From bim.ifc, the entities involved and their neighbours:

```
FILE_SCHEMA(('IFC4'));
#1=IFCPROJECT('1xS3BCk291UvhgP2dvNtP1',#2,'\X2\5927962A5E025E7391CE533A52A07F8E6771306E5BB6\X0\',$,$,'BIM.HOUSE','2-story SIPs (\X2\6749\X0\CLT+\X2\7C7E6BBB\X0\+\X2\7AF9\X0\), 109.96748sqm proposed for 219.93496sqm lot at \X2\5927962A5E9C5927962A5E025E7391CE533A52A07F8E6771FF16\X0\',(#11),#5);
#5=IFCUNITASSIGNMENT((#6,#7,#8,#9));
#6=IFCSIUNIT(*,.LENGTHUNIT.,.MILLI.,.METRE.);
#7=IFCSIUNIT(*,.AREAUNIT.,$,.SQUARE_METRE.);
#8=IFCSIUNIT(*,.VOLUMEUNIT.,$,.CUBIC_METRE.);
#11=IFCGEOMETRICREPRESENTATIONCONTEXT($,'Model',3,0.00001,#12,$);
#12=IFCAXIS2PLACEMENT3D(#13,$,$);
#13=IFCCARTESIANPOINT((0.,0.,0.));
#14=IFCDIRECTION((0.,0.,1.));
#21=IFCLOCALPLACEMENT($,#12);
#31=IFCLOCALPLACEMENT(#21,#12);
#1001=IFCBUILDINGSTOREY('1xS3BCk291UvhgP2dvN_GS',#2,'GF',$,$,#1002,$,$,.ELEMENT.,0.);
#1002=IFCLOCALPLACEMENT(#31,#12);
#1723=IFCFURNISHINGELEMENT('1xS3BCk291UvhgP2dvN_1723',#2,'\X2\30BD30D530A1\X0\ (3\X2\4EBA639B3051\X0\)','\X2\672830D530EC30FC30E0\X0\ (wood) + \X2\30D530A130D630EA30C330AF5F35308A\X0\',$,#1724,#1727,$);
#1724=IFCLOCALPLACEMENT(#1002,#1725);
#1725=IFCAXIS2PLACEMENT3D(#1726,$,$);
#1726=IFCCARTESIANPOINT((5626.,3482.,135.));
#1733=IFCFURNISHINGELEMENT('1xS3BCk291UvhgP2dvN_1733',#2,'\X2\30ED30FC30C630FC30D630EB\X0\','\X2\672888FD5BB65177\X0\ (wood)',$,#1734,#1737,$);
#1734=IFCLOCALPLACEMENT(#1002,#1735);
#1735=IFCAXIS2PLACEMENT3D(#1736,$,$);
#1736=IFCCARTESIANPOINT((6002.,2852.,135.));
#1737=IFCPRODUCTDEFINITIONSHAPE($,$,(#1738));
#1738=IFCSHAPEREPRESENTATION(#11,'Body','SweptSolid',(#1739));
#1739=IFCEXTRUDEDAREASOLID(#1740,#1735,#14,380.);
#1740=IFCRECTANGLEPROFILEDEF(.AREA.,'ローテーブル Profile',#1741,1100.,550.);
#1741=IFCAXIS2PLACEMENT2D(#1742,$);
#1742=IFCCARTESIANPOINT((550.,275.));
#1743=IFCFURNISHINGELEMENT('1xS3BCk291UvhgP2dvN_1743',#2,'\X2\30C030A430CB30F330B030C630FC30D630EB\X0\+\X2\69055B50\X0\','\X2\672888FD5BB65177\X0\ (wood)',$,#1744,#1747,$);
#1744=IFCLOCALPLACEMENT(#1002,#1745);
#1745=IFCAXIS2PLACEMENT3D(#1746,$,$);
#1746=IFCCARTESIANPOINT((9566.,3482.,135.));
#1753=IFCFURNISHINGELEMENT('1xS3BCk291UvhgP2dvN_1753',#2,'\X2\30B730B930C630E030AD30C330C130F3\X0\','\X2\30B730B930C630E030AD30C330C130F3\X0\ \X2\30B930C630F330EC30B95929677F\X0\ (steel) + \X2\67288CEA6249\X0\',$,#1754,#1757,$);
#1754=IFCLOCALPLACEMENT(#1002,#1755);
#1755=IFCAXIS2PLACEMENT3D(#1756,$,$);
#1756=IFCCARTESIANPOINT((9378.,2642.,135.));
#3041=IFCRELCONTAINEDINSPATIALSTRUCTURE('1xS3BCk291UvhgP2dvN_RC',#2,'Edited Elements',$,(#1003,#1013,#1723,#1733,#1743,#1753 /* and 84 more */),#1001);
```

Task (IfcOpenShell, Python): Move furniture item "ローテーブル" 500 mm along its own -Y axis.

```python
import ifcopenshell
import ifcopenshell.api.geometry
import ifcopenshell.util.placement
import ifcopenshell.util.unit

model = ifcopenshell.open("bim.ifc")
unit_scale = ifcopenshell.util.unit.calculate_unit_scale(model)

item = model.by_guid("1xS3BCk291UvhgP2dvN_1733")
matrix = ifcopenshell.util.placement.get_local_placement(item.ObjectPlacement)
matrix[:3, 3] -= matrix[:3, 1] * 0.5 / unit_scale
ifcopenshell.api.geometry.edit_object_placement(model, product=item, matrix=matrix, is_si=False)

print(ifcopenshell.util.placement.get_local_placement(item.ObjectPlacement).round(3) + 0.0)

model.write("bim_rev.ifc")
```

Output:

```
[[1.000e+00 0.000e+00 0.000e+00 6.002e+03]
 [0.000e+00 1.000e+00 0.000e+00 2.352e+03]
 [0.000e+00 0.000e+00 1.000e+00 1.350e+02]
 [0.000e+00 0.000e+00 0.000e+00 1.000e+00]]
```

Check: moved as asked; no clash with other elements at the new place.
